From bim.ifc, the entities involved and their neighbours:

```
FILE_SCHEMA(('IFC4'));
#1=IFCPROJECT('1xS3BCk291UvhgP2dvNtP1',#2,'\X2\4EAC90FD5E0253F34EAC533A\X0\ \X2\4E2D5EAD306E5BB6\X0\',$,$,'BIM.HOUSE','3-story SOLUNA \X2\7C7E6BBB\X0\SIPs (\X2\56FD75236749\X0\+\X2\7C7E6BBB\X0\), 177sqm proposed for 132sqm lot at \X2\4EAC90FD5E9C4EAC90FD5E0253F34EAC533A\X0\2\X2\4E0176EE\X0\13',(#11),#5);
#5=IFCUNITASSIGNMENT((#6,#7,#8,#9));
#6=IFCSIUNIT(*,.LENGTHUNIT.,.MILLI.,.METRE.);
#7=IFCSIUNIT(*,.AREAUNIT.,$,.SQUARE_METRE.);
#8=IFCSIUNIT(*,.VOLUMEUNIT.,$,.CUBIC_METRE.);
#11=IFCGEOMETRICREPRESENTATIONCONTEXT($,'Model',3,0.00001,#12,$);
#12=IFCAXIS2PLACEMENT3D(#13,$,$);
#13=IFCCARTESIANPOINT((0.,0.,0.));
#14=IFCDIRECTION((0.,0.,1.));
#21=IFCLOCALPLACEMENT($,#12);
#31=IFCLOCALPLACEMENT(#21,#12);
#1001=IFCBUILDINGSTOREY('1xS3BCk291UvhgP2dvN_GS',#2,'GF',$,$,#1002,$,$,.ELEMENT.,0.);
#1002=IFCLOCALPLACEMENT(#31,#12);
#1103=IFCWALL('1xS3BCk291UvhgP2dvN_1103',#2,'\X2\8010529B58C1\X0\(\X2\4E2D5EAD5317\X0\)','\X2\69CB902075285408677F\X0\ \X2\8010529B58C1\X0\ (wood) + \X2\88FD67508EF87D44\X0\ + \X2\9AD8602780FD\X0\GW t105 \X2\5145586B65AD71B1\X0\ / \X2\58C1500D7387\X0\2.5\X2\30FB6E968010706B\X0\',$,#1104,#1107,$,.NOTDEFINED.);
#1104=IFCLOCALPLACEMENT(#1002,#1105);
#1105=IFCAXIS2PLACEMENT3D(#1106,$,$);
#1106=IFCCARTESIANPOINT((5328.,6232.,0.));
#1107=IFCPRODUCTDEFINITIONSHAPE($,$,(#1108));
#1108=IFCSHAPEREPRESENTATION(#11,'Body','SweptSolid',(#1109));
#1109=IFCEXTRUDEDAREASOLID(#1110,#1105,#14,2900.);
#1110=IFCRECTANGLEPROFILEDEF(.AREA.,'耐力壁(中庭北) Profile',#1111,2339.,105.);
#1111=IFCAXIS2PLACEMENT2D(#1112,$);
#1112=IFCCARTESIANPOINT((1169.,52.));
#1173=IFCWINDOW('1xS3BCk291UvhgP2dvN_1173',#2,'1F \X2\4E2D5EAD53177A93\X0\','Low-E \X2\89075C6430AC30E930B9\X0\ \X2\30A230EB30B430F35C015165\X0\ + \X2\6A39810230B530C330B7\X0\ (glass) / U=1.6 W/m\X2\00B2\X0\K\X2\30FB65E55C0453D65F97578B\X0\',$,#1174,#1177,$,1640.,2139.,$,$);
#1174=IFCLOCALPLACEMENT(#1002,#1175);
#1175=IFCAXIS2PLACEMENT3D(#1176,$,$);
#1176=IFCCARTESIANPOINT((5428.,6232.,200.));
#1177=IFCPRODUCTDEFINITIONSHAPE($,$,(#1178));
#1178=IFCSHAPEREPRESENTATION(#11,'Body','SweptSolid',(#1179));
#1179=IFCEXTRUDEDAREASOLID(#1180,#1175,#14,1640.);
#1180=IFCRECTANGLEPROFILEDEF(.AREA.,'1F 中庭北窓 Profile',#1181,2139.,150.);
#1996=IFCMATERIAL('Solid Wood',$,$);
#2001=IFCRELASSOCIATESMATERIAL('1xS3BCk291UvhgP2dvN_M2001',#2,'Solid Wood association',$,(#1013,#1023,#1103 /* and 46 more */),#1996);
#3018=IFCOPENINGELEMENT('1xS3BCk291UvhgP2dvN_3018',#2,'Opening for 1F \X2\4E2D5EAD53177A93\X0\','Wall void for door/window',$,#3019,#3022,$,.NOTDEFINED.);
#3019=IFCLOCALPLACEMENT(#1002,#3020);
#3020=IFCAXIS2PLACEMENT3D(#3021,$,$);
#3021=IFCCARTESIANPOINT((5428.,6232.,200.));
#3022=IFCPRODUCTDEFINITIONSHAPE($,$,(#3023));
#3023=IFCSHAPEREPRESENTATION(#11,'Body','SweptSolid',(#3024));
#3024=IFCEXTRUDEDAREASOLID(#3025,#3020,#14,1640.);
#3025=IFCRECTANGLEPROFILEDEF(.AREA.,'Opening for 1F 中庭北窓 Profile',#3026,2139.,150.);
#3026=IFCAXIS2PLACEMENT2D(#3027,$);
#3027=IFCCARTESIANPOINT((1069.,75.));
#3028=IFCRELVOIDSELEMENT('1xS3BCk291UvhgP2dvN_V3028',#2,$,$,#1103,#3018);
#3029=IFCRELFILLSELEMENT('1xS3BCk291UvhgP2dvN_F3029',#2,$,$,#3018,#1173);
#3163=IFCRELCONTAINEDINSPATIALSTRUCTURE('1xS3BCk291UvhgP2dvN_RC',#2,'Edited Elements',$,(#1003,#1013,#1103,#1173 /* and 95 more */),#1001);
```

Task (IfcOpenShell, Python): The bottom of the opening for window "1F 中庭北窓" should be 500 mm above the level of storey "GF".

```python
import numpy as np
import ifcopenshell
import ifcopenshell.api.geometry
import ifcopenshell.geom
import ifcopenshell.util.element
import ifcopenshell.util.placement
import ifcopenshell.util.shape
import ifcopenshell.util.unit

model = ifcopenshell.open("bim.ifc")
unit_scale = ifcopenshell.util.unit.calculate_unit_scale(model)

window = model.by_guid("1xS3BCk291UvhgP2dvN_1173")
opening = window.FillsVoids[0].RelatingOpeningElement
storey = ifcopenshell.util.element.get_container(window, ifc_class="IfcBuildingStorey")
level = ifcopenshell.util.placement.get_local_placement(storey.ObjectPlacement)[2, 3]

# The opening's origin need not be at the sill, so measure its lowest point.
shape = ifcopenshell.geom.create_shape(ifcopenshell.geom.settings(), opening)
bottom = ifcopenshell.util.shape.get_shape_bottom_elevation(shape, shape.geometry) / unit_scale
dz = level + 500.0 - bottom

shift = np.array([0.0, 0.0, dz])
# The window is not placed relative to its opening, so move both.
for product in (opening, window):
    matrix = ifcopenshell.util.placement.get_local_placement(product.ObjectPlacement)
    matrix[:3, 3] += shift
    ifcopenshell.api.geometry.edit_object_placement(model, product=product, matrix=matrix, is_si=False)

print(f"moved by {dz * unit_scale:+.3f} m")

model.write("bim-out.ifc")
```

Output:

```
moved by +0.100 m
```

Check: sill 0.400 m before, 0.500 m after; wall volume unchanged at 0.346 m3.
